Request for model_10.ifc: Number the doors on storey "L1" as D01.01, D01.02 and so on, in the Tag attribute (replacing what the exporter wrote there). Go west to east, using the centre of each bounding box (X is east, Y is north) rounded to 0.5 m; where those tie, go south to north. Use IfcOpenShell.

First a look at what the model holds.

```python
import ifcopenshell
import ifcopenshell.util.element
import ifcopenshell.util.placement

model = ifcopenshell.open("model_10.ifc")
print(model.schema)
storey = next(s for s in model.by_type("IfcBuildingStorey") if s.Name == "L1")
doors = [e for e in ifcopenshell.util.element.get_decomposition(storey) if e.is_a("IfcDoor")]
for e in sorted(doors, key=lambda e: e.id()):
    origin = ifcopenshell.util.placement.get_local_placement(e.ObjectPlacement)[:3, 3]
    print(e.id(), e.Tag, e.Name, origin.round(2) + 0.0, sep=" | ")
```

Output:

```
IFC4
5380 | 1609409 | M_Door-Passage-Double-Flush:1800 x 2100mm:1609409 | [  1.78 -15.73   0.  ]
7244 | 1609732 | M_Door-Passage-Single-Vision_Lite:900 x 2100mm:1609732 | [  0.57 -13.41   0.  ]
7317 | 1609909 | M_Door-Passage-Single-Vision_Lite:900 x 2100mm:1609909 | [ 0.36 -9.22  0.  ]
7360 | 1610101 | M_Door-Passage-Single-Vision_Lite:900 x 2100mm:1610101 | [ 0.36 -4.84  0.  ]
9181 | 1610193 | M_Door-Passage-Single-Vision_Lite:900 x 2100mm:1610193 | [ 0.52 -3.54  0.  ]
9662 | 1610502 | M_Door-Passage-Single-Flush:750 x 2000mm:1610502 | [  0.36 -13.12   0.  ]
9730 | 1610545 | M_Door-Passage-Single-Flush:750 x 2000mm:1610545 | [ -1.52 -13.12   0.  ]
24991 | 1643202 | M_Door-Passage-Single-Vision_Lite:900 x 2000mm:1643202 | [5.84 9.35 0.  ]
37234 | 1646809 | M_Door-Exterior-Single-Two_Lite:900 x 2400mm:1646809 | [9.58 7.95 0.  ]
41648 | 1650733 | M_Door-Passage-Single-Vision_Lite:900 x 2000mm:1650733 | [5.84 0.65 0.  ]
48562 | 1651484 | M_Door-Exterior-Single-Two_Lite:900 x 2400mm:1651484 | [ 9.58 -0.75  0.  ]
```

```python
import ifcopenshell
import ifcopenshell.geom
import ifcopenshell.util.element
import ifcopenshell.util.shape

model = ifcopenshell.open("model_10.ifc")
settings = ifcopenshell.geom.settings()
settings.set("use-world-coords", True)


def centre(element):
    shape = ifcopenshell.geom.create_shape(settings, element)
    return ifcopenshell.util.shape.get_bbox_centroid(shape.geometry)


storey = next(s for s in model.by_type("IfcBuildingStorey") if s.Name == "L1")
doors = [e for e in ifcopenshell.util.element.get_decomposition(storey) if e.is_a("IfcDoor")]

# Insertion points can sit at a corner or the storey origin, so sort by the geometry (in metres).
centres = {e: centre(e) for e in doors}
doors.sort(key=lambda e: (round(centres[e][0] / 0.5), centres[e][1]))

for i, e in enumerate(doors, start=1):
    number = f"D01.{i:02d}"
    e.Tag = number
    print(e.id(), number)

model.write("model_10_v2.ifc")
```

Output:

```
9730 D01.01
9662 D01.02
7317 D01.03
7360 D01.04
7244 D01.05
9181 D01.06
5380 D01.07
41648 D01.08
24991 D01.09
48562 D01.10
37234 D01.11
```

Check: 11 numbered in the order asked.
